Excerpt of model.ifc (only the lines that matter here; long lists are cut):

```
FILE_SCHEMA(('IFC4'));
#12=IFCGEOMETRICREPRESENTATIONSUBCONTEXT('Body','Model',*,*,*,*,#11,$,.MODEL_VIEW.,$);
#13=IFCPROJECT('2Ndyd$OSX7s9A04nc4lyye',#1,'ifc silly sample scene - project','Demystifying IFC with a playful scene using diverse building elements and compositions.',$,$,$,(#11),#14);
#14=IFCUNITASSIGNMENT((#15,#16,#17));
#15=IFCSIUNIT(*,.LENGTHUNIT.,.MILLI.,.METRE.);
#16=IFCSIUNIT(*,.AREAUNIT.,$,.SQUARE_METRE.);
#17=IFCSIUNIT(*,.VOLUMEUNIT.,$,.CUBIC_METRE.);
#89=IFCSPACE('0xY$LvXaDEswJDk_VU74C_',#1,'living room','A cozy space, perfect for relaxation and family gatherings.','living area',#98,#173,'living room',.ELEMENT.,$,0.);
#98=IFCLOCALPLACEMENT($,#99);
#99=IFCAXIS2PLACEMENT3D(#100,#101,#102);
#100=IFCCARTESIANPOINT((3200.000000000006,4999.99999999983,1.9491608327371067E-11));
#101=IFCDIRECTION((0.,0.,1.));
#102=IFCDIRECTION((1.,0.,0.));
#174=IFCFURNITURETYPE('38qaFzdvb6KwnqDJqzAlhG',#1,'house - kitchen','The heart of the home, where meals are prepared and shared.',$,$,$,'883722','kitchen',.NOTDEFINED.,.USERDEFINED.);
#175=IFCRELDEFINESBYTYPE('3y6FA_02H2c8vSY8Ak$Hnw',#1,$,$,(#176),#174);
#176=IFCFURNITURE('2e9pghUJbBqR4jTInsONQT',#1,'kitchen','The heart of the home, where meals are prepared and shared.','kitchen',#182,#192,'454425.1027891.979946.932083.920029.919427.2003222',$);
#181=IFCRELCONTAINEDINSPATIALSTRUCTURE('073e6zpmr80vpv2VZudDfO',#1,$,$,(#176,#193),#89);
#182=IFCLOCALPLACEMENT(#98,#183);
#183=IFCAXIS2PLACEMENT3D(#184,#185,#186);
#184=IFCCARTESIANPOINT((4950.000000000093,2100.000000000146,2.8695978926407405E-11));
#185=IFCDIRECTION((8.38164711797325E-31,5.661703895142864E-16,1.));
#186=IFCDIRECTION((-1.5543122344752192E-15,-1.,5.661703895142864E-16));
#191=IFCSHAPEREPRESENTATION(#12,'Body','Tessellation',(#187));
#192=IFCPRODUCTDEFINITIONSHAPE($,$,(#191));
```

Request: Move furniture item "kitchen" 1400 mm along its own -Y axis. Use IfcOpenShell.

```python
import ifcopenshell
import ifcopenshell.api.geometry
import ifcopenshell.util.placement
import ifcopenshell.util.unit

model = ifcopenshell.open("model.ifc")
unit_scale = ifcopenshell.util.unit.calculate_unit_scale(model)

item = model.by_guid("2e9pghUJbBqR4jTInsONQT")
matrix = ifcopenshell.util.placement.get_local_placement(item.ObjectPlacement)
matrix[:3, 3] -= matrix[:3, 1] * 1.4 / unit_scale
ifcopenshell.api.geometry.edit_object_placement(model, product=item, matrix=matrix, is_si=False)

print(ifcopenshell.util.placement.get_local_placement(item.ObjectPlacement).round(3) + 0.0)

model.write("model_v2.ifc")
```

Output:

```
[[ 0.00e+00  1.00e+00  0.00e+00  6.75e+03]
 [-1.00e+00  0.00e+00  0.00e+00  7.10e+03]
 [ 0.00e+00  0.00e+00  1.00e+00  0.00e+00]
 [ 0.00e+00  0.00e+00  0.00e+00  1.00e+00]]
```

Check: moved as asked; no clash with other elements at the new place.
